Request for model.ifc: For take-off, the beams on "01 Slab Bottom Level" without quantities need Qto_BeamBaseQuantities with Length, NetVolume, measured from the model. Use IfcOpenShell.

First a look at what the model holds.

```python
import ifcopenshell
import ifcopenshell.util.element
import ifcopenshell.util.unit

model = ifcopenshell.open("model.ifc")
print(model.schema)
for unit_type in ("LENGTHUNIT", "AREAUNIT", "VOLUMEUNIT"):
    print(unit_type, ifcopenshell.util.unit.calculate_unit_scale(model, unit_type))
storey = next(s for s in model.by_type("IfcBuildingStorey") if s.Name == "01 Slab Bottom Level")
beams = [e for e in ifcopenshell.util.element.get_decomposition(storey) if e.is_a("IfcBeam")]
for e in sorted(beams, key=lambda e: e.id()):
    print(e.id(), e.is_a(), e.Name, list(ifcopenshell.util.element.get_psets(e, qtos_only=True)), sep=" | ")
```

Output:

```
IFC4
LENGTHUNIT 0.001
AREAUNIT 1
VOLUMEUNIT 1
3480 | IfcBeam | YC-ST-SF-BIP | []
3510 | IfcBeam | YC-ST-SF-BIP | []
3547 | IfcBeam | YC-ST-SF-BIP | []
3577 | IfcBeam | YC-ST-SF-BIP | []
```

```python
import ifcopenshell
import ifcopenshell.api.pset
import ifcopenshell.geom
import ifcopenshell.util.element
import ifcopenshell.util.shape
import ifcopenshell.util.unit

model = ifcopenshell.open("model.ifc")
unit_scale = ifcopenshell.util.unit.calculate_unit_scale(model)
volume_scale = ifcopenshell.util.unit.calculate_unit_scale(model, "VOLUMEUNIT")
settings = ifcopenshell.geom.settings()

storey = next(s for s in model.by_type("IfcBuildingStorey") if s.Name == "01 Slab Bottom Level")
beams = [e for e in ifcopenshell.util.element.get_decomposition(storey) if e.is_a("IfcBeam")]

for e in sorted(beams, key=lambda e: e.id()):
    if ifcopenshell.util.element.get_psets(e, qtos_only=True, should_inherit=False):
        continue
    # Geometry comes back in metres, in the element's own axes.
    shape = ifcopenshell.geom.create_shape(settings, e)
    values = {
        "Length": ifcopenshell.util.shape.get_max_xyz(shape.geometry) / unit_scale,
        "NetVolume": ifcopenshell.util.shape.get_volume(shape.geometry) / volume_scale,
    }
    qto = ifcopenshell.api.pset.add_qto(model, product=e, name="Qto_BeamBaseQuantities")
    ifcopenshell.api.pset.edit_qto(model, qto=qto, properties=values)
    print(e.id(), {k: round(v, 3) for k, v in values.items()})

model.write("model_rev.ifc")
```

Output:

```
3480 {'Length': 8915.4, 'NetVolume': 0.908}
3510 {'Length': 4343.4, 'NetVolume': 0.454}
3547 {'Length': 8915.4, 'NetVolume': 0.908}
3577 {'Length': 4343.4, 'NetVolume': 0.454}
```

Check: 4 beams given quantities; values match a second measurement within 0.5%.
